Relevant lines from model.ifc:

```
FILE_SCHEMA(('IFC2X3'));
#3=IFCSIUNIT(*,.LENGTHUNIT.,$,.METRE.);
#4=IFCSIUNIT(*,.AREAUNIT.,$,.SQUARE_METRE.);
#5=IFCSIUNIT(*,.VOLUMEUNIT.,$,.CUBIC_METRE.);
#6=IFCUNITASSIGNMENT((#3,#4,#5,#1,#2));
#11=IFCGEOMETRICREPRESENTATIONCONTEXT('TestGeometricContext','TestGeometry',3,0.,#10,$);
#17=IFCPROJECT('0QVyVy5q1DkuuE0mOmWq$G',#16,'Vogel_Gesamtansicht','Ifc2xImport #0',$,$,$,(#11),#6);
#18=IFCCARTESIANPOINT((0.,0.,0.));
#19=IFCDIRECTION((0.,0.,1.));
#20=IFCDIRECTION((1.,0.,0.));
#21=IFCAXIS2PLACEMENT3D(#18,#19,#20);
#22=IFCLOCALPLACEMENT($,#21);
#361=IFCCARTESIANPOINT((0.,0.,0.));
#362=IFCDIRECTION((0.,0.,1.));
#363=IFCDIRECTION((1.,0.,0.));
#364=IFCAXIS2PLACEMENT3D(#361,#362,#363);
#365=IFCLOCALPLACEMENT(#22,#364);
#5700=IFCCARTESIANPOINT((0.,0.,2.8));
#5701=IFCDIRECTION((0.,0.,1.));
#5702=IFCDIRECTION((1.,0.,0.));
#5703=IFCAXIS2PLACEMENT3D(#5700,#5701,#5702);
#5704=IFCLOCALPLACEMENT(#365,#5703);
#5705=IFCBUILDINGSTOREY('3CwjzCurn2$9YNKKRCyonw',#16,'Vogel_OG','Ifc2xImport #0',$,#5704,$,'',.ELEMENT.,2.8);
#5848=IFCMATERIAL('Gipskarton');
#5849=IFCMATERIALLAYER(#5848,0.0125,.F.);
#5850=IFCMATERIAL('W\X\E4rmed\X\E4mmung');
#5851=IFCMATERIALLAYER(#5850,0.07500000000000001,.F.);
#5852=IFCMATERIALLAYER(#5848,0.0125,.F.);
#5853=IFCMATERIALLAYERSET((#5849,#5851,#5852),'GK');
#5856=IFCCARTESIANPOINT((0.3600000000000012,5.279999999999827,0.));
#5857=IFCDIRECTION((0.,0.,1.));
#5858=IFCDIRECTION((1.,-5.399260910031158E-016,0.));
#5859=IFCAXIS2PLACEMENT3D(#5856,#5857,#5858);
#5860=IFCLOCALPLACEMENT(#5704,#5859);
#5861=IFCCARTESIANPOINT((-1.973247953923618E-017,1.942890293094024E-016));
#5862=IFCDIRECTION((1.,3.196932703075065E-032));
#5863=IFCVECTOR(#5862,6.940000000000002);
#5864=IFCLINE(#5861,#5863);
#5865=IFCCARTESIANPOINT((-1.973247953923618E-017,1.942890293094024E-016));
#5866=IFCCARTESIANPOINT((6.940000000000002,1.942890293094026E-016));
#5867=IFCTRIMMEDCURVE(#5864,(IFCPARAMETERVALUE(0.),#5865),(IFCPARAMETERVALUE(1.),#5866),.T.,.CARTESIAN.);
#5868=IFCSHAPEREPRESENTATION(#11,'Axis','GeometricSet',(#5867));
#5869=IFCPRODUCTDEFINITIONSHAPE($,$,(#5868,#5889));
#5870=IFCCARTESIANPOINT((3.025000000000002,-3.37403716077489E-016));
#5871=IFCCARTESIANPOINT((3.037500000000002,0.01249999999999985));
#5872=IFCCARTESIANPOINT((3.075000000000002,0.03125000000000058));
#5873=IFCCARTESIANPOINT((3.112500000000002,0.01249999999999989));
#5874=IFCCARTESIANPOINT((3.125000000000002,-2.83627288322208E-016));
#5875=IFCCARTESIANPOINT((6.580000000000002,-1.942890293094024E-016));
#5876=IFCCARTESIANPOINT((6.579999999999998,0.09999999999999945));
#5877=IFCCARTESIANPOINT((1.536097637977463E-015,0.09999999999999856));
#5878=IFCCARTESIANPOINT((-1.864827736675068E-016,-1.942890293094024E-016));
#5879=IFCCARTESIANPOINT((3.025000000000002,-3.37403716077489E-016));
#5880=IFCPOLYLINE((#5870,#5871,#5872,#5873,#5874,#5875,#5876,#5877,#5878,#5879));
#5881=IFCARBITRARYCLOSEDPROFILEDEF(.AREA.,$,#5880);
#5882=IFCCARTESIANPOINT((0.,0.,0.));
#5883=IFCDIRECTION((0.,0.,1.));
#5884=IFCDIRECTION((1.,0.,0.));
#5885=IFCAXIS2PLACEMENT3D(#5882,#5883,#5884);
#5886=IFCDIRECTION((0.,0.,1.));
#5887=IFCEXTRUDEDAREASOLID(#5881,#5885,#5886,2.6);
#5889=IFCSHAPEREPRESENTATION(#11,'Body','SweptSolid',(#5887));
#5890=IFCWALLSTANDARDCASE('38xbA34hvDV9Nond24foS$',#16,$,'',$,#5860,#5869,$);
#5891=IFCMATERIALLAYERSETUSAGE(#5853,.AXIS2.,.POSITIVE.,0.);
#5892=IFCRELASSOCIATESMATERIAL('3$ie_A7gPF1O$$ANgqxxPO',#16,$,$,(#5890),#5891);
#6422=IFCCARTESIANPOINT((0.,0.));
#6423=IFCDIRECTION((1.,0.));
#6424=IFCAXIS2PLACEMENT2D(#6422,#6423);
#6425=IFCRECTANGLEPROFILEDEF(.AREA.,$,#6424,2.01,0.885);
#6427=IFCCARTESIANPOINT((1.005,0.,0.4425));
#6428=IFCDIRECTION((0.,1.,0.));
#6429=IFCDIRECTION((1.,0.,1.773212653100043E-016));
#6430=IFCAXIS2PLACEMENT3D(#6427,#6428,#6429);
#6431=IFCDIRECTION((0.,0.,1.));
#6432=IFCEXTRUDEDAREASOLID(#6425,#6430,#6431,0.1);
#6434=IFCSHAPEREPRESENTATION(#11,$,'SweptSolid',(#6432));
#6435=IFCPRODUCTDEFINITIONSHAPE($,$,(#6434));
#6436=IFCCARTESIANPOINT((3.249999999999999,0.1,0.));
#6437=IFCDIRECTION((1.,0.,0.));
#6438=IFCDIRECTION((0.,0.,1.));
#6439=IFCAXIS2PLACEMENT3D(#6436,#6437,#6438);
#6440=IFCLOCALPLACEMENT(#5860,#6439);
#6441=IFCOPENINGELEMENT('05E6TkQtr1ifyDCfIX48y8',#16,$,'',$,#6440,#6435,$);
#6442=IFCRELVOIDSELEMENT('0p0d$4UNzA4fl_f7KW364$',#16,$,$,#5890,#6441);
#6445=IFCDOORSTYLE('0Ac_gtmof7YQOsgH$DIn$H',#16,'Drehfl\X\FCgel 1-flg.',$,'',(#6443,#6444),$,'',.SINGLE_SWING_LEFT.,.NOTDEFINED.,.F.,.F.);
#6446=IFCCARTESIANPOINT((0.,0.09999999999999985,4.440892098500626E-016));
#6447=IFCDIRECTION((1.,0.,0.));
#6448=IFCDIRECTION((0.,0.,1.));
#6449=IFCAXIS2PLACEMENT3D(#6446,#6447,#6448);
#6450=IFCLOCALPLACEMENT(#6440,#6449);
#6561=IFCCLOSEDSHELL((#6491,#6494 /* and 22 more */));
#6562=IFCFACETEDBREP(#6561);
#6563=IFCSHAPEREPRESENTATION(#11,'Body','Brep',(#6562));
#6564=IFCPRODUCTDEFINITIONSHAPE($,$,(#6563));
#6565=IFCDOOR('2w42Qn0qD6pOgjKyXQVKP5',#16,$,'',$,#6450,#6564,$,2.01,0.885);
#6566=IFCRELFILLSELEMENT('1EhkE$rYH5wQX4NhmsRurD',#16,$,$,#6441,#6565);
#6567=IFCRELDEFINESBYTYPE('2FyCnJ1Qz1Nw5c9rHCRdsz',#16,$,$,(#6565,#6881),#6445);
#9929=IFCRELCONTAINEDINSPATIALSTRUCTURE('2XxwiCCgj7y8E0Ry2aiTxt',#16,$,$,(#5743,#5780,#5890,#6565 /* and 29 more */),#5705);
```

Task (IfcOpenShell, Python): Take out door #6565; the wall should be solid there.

```python
import ifcopenshell
import ifcopenshell.api.feature
import ifcopenshell.api.root
import ifcopenshell.geom
import ifcopenshell.util.shape

model = ifcopenshell.open("model.ifc")
settings = ifcopenshell.geom.settings()


def volume(element):
    """Net volume in cubic metres, openings subtracted."""
    shape = ifcopenshell.geom.create_shape(settings, element)
    return ifcopenshell.util.shape.get_volume(shape.geometry)


door = model.by_guid("2w42Qn0qD6pOgjKyXQVKP5")
opening = door.FillsVoids[0].RelatingOpeningElement
wall = opening.VoidsElements[0].RelatingBuildingElement
before = volume(wall)

ifcopenshell.api.root.remove_product(model, product=door)
ifcopenshell.api.feature.remove_feature(model, feature=opening)

after = volume(wall)

print(f"wall volume {before:.3f} -> {after:.3f} m3")

model.write("model_v2.ifc")
```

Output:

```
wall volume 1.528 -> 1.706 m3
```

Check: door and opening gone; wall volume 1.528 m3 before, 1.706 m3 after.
